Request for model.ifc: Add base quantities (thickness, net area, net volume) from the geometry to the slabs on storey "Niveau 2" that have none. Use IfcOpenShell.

First a look at what the model holds.

```python
import ifcopenshell
import ifcopenshell.util.element
import ifcopenshell.util.unit

model = ifcopenshell.open("model.ifc")
print(model.schema)
for unit_type in ("LENGTHUNIT", "AREAUNIT", "VOLUMEUNIT"):
    print(unit_type, ifcopenshell.util.unit.calculate_unit_scale(model, unit_type))
storey = next(s for s in model.by_type("IfcBuildingStorey") if s.Name == "Niveau 2")
slabs = [e for e in ifcopenshell.util.element.get_decomposition(storey) if e.is_a("IfcSlab")]
for e in sorted(slabs, key=lambda e: e.id()):
    print(e.id(), e.is_a(), e.Name, list(ifcopenshell.util.element.get_psets(e, qtos_only=True)), sep=" | ")
```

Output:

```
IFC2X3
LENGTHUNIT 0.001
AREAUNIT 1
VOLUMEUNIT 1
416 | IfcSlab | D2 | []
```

```python
import ifcopenshell
import ifcopenshell.api.pset
import ifcopenshell.geom
import ifcopenshell.util.element
import ifcopenshell.util.shape
import ifcopenshell.util.unit

model = ifcopenshell.open("model.ifc")
unit_scale = ifcopenshell.util.unit.calculate_unit_scale(model)
area_scale = ifcopenshell.util.unit.calculate_unit_scale(model, "AREAUNIT")
volume_scale = ifcopenshell.util.unit.calculate_unit_scale(model, "VOLUMEUNIT")
settings = ifcopenshell.geom.settings()

storey = next(s for s in model.by_type("IfcBuildingStorey") if s.Name == "Niveau 2")
slabs = [e for e in ifcopenshell.util.element.get_decomposition(storey) if e.is_a("IfcSlab")]

for e in sorted(slabs, key=lambda e: e.id()):
    if ifcopenshell.util.element.get_psets(e, qtos_only=True, should_inherit=False):
        continue
    # Geometry comes back in metres, in the element's own axes.
    shape = ifcopenshell.geom.create_shape(settings, e)
    values = {
        "Width": ifcopenshell.util.shape.get_z(shape.geometry) / unit_scale,
        "NetArea": ifcopenshell.util.shape.get_footprint_area(shape.geometry) / area_scale,
        "NetVolume": ifcopenshell.util.shape.get_volume(shape.geometry) / volume_scale,
    }
    qto = ifcopenshell.api.pset.add_qto(model, product=e, name="BaseQuantities")
    ifcopenshell.api.pset.edit_qto(model, qto=qto, properties=values)
    print(e.id(), {k: round(v, 3) for k, v in values.items()})

model.write("model_updated.ifc")
```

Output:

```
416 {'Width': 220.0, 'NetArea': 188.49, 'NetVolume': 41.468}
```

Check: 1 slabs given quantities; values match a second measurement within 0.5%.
